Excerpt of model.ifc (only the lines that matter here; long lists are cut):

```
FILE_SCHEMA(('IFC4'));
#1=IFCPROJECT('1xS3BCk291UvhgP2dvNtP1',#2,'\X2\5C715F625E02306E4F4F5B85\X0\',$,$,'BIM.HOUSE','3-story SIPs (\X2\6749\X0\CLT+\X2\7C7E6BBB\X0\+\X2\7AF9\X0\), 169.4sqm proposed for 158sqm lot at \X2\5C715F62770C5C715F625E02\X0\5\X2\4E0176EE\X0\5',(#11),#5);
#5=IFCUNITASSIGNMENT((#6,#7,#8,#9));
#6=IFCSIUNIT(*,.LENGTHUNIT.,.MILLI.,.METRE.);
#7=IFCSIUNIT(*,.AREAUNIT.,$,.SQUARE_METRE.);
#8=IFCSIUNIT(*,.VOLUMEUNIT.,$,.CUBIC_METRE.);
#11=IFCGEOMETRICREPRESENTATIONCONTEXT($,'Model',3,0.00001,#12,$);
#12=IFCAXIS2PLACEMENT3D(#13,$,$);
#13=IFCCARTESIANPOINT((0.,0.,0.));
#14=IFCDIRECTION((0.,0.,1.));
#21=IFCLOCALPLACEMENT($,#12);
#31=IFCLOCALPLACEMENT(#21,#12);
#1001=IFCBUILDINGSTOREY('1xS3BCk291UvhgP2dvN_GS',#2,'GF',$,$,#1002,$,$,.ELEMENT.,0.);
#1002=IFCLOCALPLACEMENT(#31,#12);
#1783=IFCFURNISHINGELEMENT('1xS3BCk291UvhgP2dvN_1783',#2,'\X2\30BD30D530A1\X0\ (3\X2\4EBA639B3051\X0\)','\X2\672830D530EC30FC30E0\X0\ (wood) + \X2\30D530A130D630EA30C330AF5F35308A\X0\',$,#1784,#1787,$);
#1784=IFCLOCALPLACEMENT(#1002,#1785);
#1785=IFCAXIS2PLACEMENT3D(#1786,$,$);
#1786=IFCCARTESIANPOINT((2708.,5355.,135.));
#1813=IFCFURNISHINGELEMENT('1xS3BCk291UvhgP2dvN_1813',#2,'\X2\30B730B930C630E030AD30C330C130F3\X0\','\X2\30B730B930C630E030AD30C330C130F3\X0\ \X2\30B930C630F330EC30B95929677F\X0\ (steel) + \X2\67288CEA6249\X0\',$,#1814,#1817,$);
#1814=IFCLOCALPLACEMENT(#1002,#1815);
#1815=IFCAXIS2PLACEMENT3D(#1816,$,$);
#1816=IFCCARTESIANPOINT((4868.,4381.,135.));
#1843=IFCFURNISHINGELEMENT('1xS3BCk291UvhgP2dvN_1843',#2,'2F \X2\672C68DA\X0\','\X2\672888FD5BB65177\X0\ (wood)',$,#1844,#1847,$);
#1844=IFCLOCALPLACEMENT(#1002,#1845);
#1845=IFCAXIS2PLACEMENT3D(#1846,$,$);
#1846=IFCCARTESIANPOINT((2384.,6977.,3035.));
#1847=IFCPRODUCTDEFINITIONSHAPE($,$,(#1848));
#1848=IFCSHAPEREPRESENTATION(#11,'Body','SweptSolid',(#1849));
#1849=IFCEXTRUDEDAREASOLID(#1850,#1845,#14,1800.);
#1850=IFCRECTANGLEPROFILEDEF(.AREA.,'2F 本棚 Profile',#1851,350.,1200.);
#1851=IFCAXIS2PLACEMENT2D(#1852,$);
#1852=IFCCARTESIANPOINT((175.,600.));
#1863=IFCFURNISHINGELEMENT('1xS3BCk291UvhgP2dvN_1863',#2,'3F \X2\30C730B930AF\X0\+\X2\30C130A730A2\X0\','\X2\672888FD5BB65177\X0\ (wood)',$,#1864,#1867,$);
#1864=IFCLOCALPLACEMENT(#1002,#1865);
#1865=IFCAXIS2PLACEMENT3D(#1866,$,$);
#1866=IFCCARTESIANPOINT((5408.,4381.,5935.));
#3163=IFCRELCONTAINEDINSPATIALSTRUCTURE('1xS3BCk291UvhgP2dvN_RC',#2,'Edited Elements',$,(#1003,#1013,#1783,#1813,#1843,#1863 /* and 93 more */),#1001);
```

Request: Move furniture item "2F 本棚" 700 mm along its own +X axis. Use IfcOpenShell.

```python
import ifcopenshell
import ifcopenshell.api.geometry
import ifcopenshell.util.placement

model = ifcopenshell.open("model.ifc")

item = model.by_guid("1xS3BCk291UvhgP2dvN_1843")
matrix = ifcopenshell.util.placement.get_local_placement(item.ObjectPlacement)
matrix[:3, 3] += matrix[:3, 0] * 700.0
ifcopenshell.api.geometry.edit_object_placement(model, product=item, matrix=matrix, is_si=False)

print(ifcopenshell.util.placement.get_local_placement(item.ObjectPlacement).round(3) + 0.0)

model.write("model_rev.ifc")
```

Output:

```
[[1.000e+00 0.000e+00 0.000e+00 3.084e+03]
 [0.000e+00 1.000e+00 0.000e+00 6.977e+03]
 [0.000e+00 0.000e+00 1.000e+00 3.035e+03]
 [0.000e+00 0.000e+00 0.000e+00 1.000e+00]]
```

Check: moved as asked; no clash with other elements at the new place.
